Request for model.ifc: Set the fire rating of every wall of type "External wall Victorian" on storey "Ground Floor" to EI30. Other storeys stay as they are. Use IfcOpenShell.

First a look at what the model holds.

```python
import ifcopenshell
import ifcopenshell.util.element

model = ifcopenshell.open("model.ifc")
print(model.schema)
storey = next(s for s in model.by_type("IfcBuildingStorey") if s.Name == "Ground Floor")
walls = [e for e in ifcopenshell.util.element.get_decomposition(storey) if e.is_a("IfcWall")]
seen = {}
for e in walls:
    element_type = ifcopenshell.util.element.get_type(e)
    key = (element_type.Name if element_type != e and element_type else None, ifcopenshell.util.element.get_pset(e, "Pset_WallCommon", "FireRating"))
    seen[key] = seen.get(key, 0) + 1
for (name, value), count in sorted(seen.items(), key=str):
    print(count, "x", name, "|", value)
```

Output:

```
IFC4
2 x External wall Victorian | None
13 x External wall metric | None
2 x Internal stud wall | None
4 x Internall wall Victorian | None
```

```python
import ifcopenshell
import ifcopenshell.api.pset
import ifcopenshell.util.element

model = ifcopenshell.open("model.ifc")

storey = next(s for s in model.by_type("IfcBuildingStorey") if s.Name == "Ground Floor")
walls = [e for e in ifcopenshell.util.element.get_decomposition(storey) if e.is_a("IfcWall")]

count = 0
for e in walls:
    element_type = ifcopenshell.util.element.get_type(e)
    if element_type in (None, e) or element_type.Name != "External wall Victorian":
        continue
    # add_pset returns the element's existing set when there is one.
    pset = ifcopenshell.api.pset.add_pset(model, product=e, name="Pset_WallCommon")
    ifcopenshell.api.pset.edit_pset(model, pset=pset, properties={"FireRating": "EI30"})
    count += 1

print(count, "walls updated")

model.write("model_rev.ifc")
```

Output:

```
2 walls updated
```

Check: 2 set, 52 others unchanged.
